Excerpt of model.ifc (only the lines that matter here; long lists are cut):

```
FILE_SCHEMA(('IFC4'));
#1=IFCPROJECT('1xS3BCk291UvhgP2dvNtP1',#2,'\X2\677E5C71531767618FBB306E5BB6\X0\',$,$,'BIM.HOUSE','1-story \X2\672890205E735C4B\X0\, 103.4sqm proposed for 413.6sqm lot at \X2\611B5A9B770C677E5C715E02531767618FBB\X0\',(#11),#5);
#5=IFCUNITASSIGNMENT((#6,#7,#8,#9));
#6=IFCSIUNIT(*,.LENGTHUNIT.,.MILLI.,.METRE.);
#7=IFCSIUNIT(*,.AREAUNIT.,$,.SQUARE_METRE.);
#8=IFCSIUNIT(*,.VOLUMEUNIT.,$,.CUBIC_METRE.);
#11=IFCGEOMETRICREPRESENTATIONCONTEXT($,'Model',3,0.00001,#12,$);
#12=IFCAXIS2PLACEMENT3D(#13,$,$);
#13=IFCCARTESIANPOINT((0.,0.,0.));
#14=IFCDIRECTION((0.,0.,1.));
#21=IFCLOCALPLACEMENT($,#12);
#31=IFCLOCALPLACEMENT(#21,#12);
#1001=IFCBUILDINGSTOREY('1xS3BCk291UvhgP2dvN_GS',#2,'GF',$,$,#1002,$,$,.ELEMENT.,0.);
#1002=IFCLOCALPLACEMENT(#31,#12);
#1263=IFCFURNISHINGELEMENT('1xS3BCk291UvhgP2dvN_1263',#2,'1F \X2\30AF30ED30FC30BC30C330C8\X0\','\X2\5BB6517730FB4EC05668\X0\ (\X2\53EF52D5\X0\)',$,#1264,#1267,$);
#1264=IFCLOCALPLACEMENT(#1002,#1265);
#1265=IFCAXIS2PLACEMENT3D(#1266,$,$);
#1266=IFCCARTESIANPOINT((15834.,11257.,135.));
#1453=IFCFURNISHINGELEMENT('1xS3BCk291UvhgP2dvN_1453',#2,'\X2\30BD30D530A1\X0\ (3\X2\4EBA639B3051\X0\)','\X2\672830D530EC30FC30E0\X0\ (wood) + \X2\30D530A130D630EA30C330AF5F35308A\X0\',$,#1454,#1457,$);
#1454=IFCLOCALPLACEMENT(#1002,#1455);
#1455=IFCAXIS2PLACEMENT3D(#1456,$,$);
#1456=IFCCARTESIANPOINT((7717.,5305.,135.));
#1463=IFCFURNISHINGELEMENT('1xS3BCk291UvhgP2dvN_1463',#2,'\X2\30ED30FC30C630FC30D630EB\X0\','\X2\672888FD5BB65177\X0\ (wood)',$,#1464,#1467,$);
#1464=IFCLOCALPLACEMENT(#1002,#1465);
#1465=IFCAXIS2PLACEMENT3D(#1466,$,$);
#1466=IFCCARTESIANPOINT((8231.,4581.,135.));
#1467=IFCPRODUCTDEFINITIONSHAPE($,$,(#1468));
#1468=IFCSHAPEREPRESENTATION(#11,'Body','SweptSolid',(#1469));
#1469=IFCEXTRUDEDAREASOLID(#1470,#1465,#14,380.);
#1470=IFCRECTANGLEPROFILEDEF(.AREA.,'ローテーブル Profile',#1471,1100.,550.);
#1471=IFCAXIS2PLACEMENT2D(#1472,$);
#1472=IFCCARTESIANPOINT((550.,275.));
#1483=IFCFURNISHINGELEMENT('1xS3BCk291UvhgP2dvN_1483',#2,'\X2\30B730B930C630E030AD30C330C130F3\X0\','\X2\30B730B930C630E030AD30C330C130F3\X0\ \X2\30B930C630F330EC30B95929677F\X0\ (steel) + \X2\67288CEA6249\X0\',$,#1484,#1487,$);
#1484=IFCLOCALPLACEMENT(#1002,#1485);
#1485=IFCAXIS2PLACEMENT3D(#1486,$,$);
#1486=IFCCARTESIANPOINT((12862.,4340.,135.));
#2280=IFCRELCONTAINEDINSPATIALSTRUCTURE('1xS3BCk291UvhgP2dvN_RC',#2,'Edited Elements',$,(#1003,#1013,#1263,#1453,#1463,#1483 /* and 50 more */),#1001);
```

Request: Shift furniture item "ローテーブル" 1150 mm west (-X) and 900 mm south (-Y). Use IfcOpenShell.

```python
import ifcopenshell
import ifcopenshell.api.geometry
import ifcopenshell.util.placement
import ifcopenshell.util.unit

model = ifcopenshell.open("model.ifc")
unit_scale = ifcopenshell.util.unit.calculate_unit_scale(model)

item = model.by_guid("1xS3BCk291UvhgP2dvN_1463")
matrix = ifcopenshell.util.placement.get_local_placement(item.ObjectPlacement)
matrix[0, 3] -= 1.15 / unit_scale
matrix[1, 3] -= 0.9 / unit_scale
ifcopenshell.api.geometry.edit_object_placement(model, product=item, matrix=matrix, is_si=False)

print(ifcopenshell.util.placement.get_local_placement(item.ObjectPlacement).round(3) + 0.0)

model.write("model_updated.ifc")
```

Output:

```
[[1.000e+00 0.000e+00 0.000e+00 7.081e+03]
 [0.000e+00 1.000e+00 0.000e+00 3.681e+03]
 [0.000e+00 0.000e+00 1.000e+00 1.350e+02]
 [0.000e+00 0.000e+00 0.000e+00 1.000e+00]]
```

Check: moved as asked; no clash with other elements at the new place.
